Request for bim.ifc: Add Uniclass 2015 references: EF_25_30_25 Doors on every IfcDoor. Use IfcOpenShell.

First a look at what the model holds.

```python
import ifcopenshell

model = ifcopenshell.open("bim.ifc")
print(model.schema)
print("classifications:", [c.Name for c in model.by_type("IfcClassification")])
for ifc_class in ("IfcDoor", "IfcRoof", "IfcStair", "IfcWall", "IfcWindow"):
    print(ifc_class, len(model.by_type(ifc_class)))
```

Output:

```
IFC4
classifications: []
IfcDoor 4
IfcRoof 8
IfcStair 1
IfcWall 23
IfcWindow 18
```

```python
import ifcopenshell
import ifcopenshell.api.classification

model = ifcopenshell.open("bim.ifc")

system = ifcopenshell.api.classification.add_classification(model, classification="Uniclass 2015")

codes = {
    "IfcDoor": ("EF_25_30_25", "Doors"),
}
for ifc_class, (code, name) in codes.items():
    products = model.by_type(ifc_class)
    ifcopenshell.api.classification.add_reference(
        model, products=products, classification=system, identification=code, name=name
    )
    print(code, len(products))

model.write("bim_rev.ifc")
```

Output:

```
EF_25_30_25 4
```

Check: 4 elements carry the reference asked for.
